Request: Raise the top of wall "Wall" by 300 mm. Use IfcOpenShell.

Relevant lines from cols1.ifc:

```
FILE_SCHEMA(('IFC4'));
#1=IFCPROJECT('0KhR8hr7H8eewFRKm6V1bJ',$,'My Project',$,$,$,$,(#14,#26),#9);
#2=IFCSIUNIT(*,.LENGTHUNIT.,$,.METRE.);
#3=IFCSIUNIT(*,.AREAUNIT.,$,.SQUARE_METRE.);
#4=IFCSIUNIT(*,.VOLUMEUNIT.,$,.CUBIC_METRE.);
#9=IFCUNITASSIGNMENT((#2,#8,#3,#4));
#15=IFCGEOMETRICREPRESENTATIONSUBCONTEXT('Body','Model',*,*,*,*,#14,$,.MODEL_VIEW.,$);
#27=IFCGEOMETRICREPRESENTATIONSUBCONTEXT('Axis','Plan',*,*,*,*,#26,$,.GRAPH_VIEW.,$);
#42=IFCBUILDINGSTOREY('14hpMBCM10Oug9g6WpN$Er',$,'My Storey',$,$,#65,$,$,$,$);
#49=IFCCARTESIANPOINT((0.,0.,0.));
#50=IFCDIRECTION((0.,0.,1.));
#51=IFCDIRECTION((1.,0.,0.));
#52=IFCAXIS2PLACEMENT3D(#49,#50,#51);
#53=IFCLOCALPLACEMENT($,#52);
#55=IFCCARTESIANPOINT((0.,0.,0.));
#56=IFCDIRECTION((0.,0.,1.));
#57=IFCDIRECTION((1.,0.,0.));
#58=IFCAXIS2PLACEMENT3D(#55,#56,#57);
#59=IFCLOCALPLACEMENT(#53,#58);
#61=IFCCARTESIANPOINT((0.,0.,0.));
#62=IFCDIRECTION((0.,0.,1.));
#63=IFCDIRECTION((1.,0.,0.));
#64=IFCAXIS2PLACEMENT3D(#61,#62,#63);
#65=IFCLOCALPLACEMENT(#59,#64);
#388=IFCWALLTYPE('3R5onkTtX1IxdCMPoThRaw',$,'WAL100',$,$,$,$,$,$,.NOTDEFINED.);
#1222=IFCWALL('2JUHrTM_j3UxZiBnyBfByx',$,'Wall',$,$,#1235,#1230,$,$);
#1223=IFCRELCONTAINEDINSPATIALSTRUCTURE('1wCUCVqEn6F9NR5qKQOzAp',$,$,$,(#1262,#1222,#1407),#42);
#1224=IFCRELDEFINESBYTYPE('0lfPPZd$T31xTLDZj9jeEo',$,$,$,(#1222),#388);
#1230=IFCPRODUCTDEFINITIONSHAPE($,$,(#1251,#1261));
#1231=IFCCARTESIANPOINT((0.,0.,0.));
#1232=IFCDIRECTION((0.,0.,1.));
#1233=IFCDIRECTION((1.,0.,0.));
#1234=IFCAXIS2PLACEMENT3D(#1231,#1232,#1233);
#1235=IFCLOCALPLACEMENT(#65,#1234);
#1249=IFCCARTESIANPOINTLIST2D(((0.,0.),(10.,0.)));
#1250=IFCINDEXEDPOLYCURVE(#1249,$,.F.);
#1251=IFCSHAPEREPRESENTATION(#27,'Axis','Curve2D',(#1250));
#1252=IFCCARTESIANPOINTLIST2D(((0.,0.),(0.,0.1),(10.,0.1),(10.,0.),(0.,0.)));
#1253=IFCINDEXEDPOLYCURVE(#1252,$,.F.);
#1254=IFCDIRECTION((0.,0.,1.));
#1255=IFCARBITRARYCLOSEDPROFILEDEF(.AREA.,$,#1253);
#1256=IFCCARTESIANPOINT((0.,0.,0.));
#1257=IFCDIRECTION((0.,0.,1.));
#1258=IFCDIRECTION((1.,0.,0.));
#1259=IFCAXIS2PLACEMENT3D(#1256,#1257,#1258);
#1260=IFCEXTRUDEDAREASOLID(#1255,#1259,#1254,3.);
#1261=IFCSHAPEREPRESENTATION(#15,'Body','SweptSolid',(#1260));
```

```python
import ifcopenshell
import ifcopenshell.geom
import ifcopenshell.util.representation
import ifcopenshell.util.shape

model = ifcopenshell.open("cols1.ifc")
settings = ifcopenshell.geom.settings()


def volume(element):
    """Net volume in cubic metres, openings subtracted."""
    shape = ifcopenshell.geom.create_shape(settings, element)
    return ifcopenshell.util.shape.get_volume(shape.geometry)


wall = model.by_guid("2JUHrTM_j3UxZiBnyBfByx")
before = volume(wall)

body = ifcopenshell.util.representation.get_representation(wall, "Model", "Body")
solid = body.Items[0]
old_height = solid.Depth
solid.Depth += 0.3
after = volume(wall)

print(f"height {old_height:g} -> {solid.Depth:g}, volume {before:.3f} -> {after:.3f} m3")

model.write("cols1-out.ifc")
```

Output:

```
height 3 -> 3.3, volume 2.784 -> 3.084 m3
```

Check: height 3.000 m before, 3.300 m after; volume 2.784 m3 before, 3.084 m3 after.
